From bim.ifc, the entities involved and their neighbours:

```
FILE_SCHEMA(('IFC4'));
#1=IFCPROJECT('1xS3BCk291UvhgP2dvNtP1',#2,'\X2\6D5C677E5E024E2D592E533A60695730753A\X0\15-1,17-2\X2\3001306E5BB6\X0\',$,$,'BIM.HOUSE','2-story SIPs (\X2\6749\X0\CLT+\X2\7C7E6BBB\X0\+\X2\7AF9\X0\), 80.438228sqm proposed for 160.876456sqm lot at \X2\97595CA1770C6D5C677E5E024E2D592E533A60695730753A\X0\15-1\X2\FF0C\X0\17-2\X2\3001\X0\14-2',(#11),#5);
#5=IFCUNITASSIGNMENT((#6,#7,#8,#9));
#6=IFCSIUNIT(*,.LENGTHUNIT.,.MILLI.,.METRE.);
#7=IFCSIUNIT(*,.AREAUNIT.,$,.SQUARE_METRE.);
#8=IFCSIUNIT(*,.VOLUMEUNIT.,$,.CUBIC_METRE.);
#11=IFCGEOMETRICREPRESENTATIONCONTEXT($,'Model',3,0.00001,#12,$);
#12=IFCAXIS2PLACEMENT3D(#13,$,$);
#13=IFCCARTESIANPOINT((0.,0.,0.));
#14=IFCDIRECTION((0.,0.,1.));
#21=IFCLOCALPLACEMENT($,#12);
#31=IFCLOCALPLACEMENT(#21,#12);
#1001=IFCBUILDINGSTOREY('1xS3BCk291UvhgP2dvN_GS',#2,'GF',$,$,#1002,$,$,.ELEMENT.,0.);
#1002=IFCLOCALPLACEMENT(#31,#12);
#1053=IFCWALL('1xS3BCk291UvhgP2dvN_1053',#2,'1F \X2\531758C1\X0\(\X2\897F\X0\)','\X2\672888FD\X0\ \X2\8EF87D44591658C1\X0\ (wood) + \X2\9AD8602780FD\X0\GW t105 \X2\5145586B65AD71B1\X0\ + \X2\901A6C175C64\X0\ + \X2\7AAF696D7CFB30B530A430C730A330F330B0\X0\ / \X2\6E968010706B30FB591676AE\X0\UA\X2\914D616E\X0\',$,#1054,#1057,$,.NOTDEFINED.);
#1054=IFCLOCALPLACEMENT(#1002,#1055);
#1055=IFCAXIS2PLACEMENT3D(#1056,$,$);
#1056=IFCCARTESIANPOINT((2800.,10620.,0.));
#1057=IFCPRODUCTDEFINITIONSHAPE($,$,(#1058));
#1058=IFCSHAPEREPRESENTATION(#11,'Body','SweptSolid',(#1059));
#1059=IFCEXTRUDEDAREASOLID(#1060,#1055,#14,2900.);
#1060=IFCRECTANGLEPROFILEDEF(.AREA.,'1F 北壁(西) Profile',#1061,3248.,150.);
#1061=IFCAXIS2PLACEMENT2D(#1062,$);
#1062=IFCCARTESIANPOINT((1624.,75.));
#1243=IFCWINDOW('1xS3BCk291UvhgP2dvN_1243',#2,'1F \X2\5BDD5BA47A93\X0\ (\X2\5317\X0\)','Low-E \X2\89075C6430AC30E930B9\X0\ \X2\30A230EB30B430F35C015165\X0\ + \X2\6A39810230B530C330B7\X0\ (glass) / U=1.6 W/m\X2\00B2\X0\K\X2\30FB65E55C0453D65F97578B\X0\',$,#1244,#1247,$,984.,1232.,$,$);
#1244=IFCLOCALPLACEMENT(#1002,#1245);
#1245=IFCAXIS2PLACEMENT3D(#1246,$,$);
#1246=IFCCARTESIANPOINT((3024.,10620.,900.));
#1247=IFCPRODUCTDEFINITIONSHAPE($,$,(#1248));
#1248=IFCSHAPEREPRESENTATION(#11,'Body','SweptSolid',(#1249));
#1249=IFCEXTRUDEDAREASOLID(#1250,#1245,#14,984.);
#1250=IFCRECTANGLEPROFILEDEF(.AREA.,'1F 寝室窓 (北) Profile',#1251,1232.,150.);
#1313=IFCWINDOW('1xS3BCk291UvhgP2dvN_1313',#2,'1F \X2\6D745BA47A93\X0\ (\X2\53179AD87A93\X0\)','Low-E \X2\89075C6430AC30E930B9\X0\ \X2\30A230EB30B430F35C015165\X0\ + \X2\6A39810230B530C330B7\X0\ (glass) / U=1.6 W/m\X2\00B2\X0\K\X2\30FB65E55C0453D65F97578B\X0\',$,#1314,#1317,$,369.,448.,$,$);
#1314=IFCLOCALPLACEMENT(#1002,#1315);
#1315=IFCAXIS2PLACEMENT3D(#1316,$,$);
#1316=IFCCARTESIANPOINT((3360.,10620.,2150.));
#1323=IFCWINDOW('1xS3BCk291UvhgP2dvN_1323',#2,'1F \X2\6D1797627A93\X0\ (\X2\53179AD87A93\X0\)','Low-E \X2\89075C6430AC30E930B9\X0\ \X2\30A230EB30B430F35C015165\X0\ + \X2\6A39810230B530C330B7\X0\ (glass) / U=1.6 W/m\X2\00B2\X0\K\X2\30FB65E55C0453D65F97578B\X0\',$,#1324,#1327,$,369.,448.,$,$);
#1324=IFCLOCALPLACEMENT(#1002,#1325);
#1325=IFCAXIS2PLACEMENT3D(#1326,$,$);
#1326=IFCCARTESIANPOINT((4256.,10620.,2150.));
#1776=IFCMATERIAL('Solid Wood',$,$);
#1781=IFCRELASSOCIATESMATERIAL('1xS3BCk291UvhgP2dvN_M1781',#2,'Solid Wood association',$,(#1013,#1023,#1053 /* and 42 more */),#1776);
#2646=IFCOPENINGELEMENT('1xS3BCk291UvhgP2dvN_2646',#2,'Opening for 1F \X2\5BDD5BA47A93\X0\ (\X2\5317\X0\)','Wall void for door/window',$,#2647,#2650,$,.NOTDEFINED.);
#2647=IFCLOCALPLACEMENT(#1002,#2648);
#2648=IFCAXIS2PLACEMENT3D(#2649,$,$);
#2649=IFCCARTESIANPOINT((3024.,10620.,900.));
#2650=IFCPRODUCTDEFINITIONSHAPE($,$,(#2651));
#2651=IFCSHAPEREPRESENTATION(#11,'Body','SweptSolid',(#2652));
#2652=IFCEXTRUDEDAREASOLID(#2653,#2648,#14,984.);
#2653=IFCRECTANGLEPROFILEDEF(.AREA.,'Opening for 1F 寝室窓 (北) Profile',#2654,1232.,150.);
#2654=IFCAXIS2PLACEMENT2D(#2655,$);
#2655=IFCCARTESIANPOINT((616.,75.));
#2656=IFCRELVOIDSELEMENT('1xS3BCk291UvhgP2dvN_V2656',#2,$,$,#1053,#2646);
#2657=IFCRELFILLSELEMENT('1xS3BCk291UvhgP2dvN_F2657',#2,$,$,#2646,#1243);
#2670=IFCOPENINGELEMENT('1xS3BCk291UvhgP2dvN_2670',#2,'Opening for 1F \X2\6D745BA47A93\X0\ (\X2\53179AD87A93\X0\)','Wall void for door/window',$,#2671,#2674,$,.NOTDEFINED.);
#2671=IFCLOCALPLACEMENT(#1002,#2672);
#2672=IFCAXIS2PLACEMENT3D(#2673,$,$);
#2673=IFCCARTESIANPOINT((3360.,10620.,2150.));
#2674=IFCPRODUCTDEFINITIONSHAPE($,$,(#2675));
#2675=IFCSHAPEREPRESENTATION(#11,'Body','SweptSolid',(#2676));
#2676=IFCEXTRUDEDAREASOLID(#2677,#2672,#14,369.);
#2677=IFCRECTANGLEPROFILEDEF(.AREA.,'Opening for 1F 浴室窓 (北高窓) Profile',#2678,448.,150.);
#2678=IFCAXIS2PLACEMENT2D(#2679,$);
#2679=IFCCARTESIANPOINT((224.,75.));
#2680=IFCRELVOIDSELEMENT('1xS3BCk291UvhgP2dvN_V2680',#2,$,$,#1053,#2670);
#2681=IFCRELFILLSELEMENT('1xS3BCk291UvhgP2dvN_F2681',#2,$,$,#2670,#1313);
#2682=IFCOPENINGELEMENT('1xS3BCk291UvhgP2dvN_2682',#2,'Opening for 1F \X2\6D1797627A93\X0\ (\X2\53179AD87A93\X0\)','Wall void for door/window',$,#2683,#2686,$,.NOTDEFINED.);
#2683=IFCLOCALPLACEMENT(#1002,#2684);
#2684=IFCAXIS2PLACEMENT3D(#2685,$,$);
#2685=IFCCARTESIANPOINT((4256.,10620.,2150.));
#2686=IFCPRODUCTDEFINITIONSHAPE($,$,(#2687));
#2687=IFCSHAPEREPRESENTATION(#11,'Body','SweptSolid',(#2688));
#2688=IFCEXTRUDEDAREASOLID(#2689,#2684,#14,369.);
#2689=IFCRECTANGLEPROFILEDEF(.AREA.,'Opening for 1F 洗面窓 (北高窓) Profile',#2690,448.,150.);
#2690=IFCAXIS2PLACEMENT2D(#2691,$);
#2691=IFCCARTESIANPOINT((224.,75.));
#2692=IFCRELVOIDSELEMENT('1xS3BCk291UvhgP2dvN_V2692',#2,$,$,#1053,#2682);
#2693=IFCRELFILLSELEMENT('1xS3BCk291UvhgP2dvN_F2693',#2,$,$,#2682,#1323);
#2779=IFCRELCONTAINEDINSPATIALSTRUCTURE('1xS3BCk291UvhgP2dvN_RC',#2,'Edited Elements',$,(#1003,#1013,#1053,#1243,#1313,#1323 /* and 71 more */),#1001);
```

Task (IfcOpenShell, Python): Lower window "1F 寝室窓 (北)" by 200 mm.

```python
import numpy as np
import ifcopenshell
import ifcopenshell.api.geometry
import ifcopenshell.util.placement
import ifcopenshell.util.unit

model = ifcopenshell.open("bim.ifc")
unit_scale = ifcopenshell.util.unit.calculate_unit_scale(model)

window = model.by_guid("1xS3BCk291UvhgP2dvN_1243")
opening = window.FillsVoids[0].RelatingOpeningElement
dz = -0.2 / unit_scale

shift = np.array([0.0, 0.0, dz])
# The window is not placed relative to its opening, so move both.
for product in (opening, window):
    matrix = ifcopenshell.util.placement.get_local_placement(product.ObjectPlacement)
    matrix[:3, 3] += shift
    ifcopenshell.api.geometry.edit_object_placement(model, product=product, matrix=matrix, is_si=False)

print(f"moved by {dz * unit_scale:+.3f} m")

model.write("bim_rev.ifc")
```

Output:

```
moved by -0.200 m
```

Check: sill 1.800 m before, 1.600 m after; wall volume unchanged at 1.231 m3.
